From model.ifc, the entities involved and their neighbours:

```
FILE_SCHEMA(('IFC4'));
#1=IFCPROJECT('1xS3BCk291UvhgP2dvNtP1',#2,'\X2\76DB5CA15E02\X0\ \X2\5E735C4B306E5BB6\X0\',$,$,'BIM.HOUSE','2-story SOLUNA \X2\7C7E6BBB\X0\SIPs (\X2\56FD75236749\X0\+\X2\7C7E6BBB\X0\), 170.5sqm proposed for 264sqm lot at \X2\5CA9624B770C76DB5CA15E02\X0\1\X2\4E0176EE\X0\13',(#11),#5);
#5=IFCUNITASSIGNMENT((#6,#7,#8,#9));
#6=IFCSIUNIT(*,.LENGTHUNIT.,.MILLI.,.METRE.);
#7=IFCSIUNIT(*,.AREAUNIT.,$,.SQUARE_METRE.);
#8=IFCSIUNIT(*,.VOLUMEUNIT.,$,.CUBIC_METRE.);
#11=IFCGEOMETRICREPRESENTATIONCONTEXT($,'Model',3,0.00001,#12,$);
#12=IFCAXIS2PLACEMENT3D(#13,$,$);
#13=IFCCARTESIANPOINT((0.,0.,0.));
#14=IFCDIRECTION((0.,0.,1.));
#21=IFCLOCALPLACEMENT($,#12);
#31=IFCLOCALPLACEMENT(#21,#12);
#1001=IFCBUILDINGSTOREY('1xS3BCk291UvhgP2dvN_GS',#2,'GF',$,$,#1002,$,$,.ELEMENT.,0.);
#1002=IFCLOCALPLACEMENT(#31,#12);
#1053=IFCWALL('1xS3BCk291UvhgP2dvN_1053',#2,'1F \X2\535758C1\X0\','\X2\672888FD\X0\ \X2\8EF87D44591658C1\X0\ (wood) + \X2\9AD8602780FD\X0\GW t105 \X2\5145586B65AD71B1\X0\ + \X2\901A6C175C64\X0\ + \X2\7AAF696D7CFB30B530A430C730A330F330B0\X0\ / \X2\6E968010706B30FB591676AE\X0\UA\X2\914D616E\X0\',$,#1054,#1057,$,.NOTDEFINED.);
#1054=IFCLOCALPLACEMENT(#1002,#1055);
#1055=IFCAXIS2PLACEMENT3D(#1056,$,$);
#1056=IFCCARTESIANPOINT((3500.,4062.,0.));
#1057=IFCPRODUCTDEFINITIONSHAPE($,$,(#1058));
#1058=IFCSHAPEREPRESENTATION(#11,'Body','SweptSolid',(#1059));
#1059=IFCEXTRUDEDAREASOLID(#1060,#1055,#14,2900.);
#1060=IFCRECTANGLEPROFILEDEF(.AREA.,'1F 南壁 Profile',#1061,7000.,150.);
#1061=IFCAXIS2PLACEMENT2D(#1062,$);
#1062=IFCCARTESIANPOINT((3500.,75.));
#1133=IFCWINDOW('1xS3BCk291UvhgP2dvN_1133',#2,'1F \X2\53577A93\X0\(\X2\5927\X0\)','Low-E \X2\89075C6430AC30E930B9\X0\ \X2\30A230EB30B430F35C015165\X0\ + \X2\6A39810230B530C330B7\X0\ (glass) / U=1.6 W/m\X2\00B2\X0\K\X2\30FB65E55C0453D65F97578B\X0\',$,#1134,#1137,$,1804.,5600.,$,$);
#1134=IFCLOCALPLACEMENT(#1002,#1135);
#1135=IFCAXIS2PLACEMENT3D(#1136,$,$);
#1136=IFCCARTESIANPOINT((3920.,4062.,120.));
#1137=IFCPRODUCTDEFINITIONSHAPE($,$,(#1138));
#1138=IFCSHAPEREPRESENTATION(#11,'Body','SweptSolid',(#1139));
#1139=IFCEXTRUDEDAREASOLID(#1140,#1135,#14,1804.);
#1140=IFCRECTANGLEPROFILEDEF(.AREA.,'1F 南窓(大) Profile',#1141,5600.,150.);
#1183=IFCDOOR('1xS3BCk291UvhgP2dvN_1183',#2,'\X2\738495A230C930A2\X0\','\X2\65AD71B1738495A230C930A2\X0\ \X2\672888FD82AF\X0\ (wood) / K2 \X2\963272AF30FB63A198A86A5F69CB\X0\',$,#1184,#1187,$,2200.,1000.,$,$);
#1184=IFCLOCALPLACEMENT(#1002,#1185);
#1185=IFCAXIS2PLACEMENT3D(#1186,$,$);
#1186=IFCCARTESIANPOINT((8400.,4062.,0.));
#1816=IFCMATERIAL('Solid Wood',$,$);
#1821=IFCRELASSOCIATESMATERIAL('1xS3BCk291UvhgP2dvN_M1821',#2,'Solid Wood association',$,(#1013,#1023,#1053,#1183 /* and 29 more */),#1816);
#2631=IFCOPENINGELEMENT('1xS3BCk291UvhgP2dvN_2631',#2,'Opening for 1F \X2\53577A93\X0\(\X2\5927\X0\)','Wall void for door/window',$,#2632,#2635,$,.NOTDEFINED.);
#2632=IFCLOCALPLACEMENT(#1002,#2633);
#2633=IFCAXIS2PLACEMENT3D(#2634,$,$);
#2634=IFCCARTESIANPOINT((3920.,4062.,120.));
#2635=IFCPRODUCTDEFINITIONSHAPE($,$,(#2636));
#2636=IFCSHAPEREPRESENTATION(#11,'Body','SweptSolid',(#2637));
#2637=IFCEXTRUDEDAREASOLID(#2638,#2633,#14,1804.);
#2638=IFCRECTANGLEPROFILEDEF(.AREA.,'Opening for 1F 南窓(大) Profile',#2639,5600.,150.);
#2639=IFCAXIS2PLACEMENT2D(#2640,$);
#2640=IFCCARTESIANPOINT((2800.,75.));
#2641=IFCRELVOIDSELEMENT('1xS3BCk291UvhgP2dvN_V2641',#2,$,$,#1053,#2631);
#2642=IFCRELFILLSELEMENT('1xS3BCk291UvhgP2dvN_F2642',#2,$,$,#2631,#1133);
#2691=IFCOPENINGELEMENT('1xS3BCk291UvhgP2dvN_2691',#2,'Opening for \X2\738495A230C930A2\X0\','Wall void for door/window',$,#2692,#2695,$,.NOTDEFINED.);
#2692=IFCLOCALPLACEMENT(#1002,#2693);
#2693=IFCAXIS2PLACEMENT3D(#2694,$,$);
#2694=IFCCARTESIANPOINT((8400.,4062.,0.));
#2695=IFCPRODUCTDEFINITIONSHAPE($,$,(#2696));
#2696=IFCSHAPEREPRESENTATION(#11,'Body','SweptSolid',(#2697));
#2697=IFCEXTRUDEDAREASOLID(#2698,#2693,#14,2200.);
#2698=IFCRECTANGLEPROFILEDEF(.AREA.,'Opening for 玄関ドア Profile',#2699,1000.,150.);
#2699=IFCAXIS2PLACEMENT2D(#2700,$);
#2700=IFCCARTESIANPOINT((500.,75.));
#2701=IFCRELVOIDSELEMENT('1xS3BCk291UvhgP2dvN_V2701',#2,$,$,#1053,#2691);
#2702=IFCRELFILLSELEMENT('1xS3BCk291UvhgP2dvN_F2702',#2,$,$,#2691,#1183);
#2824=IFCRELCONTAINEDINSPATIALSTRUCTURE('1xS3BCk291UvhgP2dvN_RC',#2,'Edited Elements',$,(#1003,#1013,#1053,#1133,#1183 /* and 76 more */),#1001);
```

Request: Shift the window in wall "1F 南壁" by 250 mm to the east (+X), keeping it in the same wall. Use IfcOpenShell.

```python
import ifcopenshell
import ifcopenshell.api.geometry
import ifcopenshell.util.placement
import ifcopenshell.util.unit

model = ifcopenshell.open("model.ifc")
unit_scale = ifcopenshell.util.unit.calculate_unit_scale(model)

window = model.by_id(1133)
opening = window.FillsVoids[0].RelatingOpeningElement
wall = opening.VoidsElements[0].RelatingBuildingElement

wall_matrix = ifcopenshell.util.placement.get_local_placement(wall.ObjectPlacement)
shift = wall_matrix[:3, 0] * 0.25 / unit_scale
before = ifcopenshell.util.placement.get_local_placement(window.ObjectPlacement)[:3, 3].copy()

# The window is not placed relative to its opening, so move both.
for product in (opening, window):
    matrix = ifcopenshell.util.placement.get_local_placement(product.ObjectPlacement)
    matrix[:3, 3] += shift
    ifcopenshell.api.geometry.edit_object_placement(model, product=product, matrix=matrix, is_si=False)

after = ifcopenshell.util.placement.get_local_placement(window.ObjectPlacement)[:3, 3]
print("window moved by", (after - before).round(3) + 0.0)

model.write("model_edited.ifc")
```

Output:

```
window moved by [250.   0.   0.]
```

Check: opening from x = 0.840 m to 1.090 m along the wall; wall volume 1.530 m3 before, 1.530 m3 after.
